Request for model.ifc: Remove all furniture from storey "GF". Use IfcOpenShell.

First a look at what the model holds.

```python
import ifcopenshell
import ifcopenshell.util.element

model = ifcopenshell.open("model.ifc")
print(model.schema)
storey = next(s for s in model.by_type("IfcBuildingStorey") if s.Name == "GF")
furniture = [e for e in ifcopenshell.util.element.get_decomposition(storey) if e.is_a("IfcFurnishingElement")]
seen = {}
for e in furniture:
    element_type = ifcopenshell.util.element.get_type(e)
    name = element_type.Name if element_type not in (None, e) else None
    seen[name] = seen.get(name, 0) + 1
for name, count in sorted(seen.items(), key=str):
    print(count, "x", name)
```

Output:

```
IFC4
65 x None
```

```python
import ifcopenshell
import ifcopenshell.api.root
import ifcopenshell.util.element

model = ifcopenshell.open("model.ifc")

storey = next(s for s in model.by_type("IfcBuildingStorey") if s.Name == "GF")
furniture = [e for e in ifcopenshell.util.element.get_decomposition(storey) if e.is_a("IfcFurnishingElement")]

for e in furniture:
    ifcopenshell.api.root.remove_product(model, product=e)
print(len(furniture), "removed")

model.write("model_rev.ifc")
```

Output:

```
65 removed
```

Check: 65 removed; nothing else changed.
